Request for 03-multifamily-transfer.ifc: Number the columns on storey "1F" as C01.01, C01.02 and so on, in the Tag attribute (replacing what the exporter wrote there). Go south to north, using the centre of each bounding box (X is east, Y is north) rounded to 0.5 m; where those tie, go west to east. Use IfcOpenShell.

First a look at what the model holds.

```python
import ifcopenshell
import ifcopenshell.util.element
import ifcopenshell.util.placement

model = ifcopenshell.open("03-multifamily-transfer.ifc")
print(model.schema)
storey = next(s for s in model.by_type("IfcBuildingStorey") if s.Name == "1F")
columns = [e for e in ifcopenshell.util.element.get_decomposition(storey) if e.is_a("IfcColumn")]
for e in sorted(columns, key=lambda e: e.id()):
    origin = ifcopenshell.util.placement.get_local_placement(e.ObjectPlacement)[:3, 3]
    print(e.id(), e.Tag, e.Name, origin.round(2) + 0.0, sep=" | ")
```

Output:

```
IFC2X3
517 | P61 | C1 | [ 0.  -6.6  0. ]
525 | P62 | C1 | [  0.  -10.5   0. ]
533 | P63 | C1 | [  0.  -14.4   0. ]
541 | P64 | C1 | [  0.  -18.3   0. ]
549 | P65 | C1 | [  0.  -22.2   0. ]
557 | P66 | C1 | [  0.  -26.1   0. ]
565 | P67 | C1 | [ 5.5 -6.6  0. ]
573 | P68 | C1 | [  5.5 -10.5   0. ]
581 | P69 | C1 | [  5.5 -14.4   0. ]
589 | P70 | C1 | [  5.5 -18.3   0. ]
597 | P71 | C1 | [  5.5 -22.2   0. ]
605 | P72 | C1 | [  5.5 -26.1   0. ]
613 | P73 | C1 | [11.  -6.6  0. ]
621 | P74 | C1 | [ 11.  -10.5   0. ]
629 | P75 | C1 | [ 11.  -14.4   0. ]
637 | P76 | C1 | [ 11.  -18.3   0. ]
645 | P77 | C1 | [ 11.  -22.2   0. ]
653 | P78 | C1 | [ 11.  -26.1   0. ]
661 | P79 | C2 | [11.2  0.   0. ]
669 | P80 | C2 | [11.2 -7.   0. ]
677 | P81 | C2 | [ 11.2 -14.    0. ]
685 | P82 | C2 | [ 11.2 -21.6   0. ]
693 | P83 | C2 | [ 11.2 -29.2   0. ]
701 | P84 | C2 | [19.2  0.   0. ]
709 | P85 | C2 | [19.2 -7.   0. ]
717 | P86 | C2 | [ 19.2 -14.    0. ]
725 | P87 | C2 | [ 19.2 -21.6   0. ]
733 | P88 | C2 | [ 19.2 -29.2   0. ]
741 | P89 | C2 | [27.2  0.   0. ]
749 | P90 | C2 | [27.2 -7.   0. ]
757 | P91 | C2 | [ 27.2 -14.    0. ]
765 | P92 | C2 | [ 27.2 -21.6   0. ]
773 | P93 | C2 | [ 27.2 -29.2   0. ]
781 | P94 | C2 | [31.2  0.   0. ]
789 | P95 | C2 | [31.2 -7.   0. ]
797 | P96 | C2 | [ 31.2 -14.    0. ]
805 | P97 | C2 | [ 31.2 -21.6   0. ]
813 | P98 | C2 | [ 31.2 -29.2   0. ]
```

```python
import ifcopenshell
import ifcopenshell.geom
import ifcopenshell.util.element
import ifcopenshell.util.shape

model = ifcopenshell.open("03-multifamily-transfer.ifc")
settings = ifcopenshell.geom.settings()
settings.set("use-world-coords", True)


def centre(element):
    shape = ifcopenshell.geom.create_shape(settings, element)
    return ifcopenshell.util.shape.get_bbox_centroid(shape.geometry)


storey = next(s for s in model.by_type("IfcBuildingStorey") if s.Name == "1F")
columns = [e for e in ifcopenshell.util.element.get_decomposition(storey) if e.is_a("IfcColumn")]

# Insertion points can sit at a corner or the storey origin, so sort by the geometry (in metres).
centres = {e: centre(e) for e in columns}
columns.sort(key=lambda e: (round(centres[e][1] / 0.5), centres[e][0]))

for i, e in enumerate(columns, start=1):
    number = f"C01.{i:02d}"
    e.Tag = number
    print(e.id(), number)

model.write("03-multifamily-transfer-out.ifc")
```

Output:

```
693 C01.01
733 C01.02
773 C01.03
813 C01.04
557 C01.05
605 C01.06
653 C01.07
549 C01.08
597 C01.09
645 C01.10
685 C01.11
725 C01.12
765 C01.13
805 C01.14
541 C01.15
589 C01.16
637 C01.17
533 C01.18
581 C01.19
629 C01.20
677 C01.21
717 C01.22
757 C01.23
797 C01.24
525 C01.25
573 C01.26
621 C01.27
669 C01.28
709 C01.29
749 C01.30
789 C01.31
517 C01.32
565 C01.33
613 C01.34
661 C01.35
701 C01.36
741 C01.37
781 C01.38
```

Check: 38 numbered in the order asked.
